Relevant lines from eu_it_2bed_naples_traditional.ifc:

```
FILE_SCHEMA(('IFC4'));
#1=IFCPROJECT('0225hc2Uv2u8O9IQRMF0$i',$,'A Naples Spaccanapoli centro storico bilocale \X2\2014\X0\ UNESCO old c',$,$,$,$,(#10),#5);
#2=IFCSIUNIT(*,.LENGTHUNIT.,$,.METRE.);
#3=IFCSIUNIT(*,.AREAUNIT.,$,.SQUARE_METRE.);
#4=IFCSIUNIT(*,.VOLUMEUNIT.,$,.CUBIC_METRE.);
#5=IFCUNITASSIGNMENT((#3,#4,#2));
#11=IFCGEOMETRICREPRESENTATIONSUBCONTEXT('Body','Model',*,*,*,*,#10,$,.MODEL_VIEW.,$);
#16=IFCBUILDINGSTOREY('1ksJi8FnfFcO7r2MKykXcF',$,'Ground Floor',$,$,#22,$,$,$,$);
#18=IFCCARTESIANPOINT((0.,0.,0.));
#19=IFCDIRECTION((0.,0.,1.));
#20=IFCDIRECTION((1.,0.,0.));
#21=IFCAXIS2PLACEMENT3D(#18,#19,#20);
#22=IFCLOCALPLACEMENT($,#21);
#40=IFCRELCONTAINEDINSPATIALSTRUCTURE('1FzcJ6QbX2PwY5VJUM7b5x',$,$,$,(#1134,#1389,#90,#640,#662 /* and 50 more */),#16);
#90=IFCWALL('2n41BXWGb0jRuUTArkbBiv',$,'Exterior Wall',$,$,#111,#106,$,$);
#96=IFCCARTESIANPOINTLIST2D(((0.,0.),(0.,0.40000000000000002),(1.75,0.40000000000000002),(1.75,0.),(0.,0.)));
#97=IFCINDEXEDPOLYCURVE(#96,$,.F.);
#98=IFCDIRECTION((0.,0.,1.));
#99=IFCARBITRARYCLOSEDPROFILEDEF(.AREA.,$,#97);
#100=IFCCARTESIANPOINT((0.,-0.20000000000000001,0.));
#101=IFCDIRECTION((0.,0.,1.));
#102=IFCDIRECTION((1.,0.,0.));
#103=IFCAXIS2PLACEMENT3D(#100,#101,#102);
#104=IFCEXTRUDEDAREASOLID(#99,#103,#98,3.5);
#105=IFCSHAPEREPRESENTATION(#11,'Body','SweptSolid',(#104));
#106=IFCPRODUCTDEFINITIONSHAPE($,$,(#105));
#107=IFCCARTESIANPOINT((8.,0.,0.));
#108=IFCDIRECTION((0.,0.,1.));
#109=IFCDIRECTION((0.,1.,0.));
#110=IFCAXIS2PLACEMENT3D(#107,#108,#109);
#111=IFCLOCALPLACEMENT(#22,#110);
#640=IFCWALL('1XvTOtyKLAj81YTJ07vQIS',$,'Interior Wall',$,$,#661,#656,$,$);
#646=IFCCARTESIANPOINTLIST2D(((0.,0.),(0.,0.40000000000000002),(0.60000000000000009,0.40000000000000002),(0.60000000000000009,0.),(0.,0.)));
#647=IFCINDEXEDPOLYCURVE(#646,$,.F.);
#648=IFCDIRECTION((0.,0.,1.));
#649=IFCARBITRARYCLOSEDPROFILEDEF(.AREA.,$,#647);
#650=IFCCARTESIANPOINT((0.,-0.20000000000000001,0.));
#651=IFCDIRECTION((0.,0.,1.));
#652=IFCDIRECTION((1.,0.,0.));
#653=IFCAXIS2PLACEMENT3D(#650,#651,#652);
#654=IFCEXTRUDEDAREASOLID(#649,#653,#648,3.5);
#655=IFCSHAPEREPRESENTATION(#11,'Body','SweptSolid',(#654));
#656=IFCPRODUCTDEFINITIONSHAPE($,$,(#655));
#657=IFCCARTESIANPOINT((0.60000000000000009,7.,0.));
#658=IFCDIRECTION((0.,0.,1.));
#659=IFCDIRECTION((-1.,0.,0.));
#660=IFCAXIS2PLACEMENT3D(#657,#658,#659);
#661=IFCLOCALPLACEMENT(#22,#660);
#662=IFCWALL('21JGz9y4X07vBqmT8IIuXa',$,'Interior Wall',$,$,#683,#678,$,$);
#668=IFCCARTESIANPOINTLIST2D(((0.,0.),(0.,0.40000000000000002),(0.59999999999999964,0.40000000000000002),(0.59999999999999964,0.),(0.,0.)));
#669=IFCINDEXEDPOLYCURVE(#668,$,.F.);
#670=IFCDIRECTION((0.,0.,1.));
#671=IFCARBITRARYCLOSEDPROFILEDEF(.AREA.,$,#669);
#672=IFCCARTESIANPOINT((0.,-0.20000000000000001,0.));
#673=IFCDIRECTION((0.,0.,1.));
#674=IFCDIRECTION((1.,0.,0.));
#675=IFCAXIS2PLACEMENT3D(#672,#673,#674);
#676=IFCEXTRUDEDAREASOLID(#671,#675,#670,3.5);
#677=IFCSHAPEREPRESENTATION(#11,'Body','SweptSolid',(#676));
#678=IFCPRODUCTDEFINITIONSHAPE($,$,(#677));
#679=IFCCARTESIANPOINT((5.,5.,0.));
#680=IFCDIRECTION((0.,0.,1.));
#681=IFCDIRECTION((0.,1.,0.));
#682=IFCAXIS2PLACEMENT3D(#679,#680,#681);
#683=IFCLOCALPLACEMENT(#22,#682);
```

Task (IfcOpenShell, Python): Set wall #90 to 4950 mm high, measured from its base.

```python
import ifcopenshell
import ifcopenshell.geom
import ifcopenshell.util.representation
import ifcopenshell.util.shape
import ifcopenshell.util.unit

model = ifcopenshell.open("eu_it_2bed_naples_traditional.ifc")
unit_scale = ifcopenshell.util.unit.calculate_unit_scale(model)
settings = ifcopenshell.geom.settings()


def volume(element):
    """Net volume in cubic metres, openings subtracted."""
    shape = ifcopenshell.geom.create_shape(settings, element)
    return ifcopenshell.util.shape.get_volume(shape.geometry)


wall = model.by_guid("2n41BXWGb0jRuUTArkbBiv")
before = volume(wall)

body = ifcopenshell.util.representation.get_representation(wall, "Model", "Body")
solid = body.Items[0]
old_height = solid.Depth
solid.Depth = 4.95 / unit_scale
after = volume(wall)

print(f"height {old_height:g} -> {solid.Depth:g}, volume {before:.3f} -> {after:.3f} m3")

model.write("eu_it_2bed_naples_traditional_updated.ifc")
```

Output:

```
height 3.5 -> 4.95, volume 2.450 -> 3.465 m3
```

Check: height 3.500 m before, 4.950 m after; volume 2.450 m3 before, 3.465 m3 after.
